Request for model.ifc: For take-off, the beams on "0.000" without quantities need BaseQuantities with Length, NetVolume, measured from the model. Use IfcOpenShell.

First a look at what the model holds.

```python
import ifcopenshell
import ifcopenshell.util.element
import ifcopenshell.util.unit

model = ifcopenshell.open("model.ifc")
print(model.schema)
for unit_type in ("LENGTHUNIT", "AREAUNIT", "VOLUMEUNIT"):
    print(unit_type, ifcopenshell.util.unit.calculate_unit_scale(model, unit_type))
storey = next(s for s in model.by_type("IfcBuildingStorey") if s.Name == "0.000")
beams = [e for e in ifcopenshell.util.element.get_decomposition(storey) if e.is_a("IfcBeam")]
for e in sorted(beams, key=lambda e: e.id()):
    print(e.id(), e.is_a(), e.Name, list(ifcopenshell.util.element.get_psets(e, qtos_only=True)), sep=" | ")
```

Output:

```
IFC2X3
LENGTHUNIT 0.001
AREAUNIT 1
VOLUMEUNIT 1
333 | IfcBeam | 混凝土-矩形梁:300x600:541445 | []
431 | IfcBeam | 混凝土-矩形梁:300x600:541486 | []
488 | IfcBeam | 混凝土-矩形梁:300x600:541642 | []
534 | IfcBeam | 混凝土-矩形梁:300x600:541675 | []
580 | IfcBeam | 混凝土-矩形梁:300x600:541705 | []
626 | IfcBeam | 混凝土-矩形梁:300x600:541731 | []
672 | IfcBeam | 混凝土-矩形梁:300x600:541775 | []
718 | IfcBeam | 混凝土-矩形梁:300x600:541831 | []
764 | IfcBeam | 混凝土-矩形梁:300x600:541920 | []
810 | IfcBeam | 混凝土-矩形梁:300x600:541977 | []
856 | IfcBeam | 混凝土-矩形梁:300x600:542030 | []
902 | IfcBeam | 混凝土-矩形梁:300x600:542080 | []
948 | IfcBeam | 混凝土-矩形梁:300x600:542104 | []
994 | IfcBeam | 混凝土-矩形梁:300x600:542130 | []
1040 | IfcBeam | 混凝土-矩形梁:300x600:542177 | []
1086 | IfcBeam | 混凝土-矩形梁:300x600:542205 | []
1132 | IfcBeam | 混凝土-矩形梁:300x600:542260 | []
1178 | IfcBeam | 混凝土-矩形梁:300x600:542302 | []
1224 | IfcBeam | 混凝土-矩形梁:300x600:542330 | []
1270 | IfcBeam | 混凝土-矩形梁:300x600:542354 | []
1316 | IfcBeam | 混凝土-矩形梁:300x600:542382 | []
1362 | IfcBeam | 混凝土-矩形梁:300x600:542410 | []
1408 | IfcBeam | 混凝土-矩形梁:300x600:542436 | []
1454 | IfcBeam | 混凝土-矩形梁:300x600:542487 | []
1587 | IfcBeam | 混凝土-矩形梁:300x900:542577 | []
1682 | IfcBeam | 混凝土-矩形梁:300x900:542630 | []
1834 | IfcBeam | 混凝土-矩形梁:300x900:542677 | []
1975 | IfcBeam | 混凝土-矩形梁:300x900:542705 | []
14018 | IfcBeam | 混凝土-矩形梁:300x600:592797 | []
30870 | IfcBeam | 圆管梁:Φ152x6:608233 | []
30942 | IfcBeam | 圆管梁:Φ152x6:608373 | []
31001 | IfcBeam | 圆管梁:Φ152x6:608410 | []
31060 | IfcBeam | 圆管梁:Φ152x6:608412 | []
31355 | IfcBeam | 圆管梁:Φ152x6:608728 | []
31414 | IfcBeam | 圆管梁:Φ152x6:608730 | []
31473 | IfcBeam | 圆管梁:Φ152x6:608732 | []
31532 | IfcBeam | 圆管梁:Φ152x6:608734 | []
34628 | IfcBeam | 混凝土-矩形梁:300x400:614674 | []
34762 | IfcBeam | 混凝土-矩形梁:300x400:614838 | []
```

```python
import ifcopenshell
import ifcopenshell.api.pset
import ifcopenshell.geom
import ifcopenshell.util.element
import ifcopenshell.util.shape
import ifcopenshell.util.unit

model = ifcopenshell.open("model.ifc")
unit_scale = ifcopenshell.util.unit.calculate_unit_scale(model)
volume_scale = ifcopenshell.util.unit.calculate_unit_scale(model, "VOLUMEUNIT")
settings = ifcopenshell.geom.settings()

storey = next(s for s in model.by_type("IfcBuildingStorey") if s.Name == "0.000")
beams = [e for e in ifcopenshell.util.element.get_decomposition(storey) if e.is_a("IfcBeam")]

for e in sorted(beams, key=lambda e: e.id()):
    if ifcopenshell.util.element.get_psets(e, qtos_only=True, should_inherit=False):
        continue
    # Geometry comes back in metres, in the element's own axes.
    shape = ifcopenshell.geom.create_shape(settings, e)
    values = {
        "Length": ifcopenshell.util.shape.get_max_xyz(shape.geometry) / unit_scale,
        "NetVolume": ifcopenshell.util.shape.get_volume(shape.geometry) / volume_scale,
    }
    qto = ifcopenshell.api.pset.add_qto(model, product=e, name="BaseQuantities")
    ifcopenshell.api.pset.edit_qto(model, qto=qto, properties=values)
    print(e.id(), {k: round(v, 3) for k, v in values.items()})

model.write("model_edited.ifc")
```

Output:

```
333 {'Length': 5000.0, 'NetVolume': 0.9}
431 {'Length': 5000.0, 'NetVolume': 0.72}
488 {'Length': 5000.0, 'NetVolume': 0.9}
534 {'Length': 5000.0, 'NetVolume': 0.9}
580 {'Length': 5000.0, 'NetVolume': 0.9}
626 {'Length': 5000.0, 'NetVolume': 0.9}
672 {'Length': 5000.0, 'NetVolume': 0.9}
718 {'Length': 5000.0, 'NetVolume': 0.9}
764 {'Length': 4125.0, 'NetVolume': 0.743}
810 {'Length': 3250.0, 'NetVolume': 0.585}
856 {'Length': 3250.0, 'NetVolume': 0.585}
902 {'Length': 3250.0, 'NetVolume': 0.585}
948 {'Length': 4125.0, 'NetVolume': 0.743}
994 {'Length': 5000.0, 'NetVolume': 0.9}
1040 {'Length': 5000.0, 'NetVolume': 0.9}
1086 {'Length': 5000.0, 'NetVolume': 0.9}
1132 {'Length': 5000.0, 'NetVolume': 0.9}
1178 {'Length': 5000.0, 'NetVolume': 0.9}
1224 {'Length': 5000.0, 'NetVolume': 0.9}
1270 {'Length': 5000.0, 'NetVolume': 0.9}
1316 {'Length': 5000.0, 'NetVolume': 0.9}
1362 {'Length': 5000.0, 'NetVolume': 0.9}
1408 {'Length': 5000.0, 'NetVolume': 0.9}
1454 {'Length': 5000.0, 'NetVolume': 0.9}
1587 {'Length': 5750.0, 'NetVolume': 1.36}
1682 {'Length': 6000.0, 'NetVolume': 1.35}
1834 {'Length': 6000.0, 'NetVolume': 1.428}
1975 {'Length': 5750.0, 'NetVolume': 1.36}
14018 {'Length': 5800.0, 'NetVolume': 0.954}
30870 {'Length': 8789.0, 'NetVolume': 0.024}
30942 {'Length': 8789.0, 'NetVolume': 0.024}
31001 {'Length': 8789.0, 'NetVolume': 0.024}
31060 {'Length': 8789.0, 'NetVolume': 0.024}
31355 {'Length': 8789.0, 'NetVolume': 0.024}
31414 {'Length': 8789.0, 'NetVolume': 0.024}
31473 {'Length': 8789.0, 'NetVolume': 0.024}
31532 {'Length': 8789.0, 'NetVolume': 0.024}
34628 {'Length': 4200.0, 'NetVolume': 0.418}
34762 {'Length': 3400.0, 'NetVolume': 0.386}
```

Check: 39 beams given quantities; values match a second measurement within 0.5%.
